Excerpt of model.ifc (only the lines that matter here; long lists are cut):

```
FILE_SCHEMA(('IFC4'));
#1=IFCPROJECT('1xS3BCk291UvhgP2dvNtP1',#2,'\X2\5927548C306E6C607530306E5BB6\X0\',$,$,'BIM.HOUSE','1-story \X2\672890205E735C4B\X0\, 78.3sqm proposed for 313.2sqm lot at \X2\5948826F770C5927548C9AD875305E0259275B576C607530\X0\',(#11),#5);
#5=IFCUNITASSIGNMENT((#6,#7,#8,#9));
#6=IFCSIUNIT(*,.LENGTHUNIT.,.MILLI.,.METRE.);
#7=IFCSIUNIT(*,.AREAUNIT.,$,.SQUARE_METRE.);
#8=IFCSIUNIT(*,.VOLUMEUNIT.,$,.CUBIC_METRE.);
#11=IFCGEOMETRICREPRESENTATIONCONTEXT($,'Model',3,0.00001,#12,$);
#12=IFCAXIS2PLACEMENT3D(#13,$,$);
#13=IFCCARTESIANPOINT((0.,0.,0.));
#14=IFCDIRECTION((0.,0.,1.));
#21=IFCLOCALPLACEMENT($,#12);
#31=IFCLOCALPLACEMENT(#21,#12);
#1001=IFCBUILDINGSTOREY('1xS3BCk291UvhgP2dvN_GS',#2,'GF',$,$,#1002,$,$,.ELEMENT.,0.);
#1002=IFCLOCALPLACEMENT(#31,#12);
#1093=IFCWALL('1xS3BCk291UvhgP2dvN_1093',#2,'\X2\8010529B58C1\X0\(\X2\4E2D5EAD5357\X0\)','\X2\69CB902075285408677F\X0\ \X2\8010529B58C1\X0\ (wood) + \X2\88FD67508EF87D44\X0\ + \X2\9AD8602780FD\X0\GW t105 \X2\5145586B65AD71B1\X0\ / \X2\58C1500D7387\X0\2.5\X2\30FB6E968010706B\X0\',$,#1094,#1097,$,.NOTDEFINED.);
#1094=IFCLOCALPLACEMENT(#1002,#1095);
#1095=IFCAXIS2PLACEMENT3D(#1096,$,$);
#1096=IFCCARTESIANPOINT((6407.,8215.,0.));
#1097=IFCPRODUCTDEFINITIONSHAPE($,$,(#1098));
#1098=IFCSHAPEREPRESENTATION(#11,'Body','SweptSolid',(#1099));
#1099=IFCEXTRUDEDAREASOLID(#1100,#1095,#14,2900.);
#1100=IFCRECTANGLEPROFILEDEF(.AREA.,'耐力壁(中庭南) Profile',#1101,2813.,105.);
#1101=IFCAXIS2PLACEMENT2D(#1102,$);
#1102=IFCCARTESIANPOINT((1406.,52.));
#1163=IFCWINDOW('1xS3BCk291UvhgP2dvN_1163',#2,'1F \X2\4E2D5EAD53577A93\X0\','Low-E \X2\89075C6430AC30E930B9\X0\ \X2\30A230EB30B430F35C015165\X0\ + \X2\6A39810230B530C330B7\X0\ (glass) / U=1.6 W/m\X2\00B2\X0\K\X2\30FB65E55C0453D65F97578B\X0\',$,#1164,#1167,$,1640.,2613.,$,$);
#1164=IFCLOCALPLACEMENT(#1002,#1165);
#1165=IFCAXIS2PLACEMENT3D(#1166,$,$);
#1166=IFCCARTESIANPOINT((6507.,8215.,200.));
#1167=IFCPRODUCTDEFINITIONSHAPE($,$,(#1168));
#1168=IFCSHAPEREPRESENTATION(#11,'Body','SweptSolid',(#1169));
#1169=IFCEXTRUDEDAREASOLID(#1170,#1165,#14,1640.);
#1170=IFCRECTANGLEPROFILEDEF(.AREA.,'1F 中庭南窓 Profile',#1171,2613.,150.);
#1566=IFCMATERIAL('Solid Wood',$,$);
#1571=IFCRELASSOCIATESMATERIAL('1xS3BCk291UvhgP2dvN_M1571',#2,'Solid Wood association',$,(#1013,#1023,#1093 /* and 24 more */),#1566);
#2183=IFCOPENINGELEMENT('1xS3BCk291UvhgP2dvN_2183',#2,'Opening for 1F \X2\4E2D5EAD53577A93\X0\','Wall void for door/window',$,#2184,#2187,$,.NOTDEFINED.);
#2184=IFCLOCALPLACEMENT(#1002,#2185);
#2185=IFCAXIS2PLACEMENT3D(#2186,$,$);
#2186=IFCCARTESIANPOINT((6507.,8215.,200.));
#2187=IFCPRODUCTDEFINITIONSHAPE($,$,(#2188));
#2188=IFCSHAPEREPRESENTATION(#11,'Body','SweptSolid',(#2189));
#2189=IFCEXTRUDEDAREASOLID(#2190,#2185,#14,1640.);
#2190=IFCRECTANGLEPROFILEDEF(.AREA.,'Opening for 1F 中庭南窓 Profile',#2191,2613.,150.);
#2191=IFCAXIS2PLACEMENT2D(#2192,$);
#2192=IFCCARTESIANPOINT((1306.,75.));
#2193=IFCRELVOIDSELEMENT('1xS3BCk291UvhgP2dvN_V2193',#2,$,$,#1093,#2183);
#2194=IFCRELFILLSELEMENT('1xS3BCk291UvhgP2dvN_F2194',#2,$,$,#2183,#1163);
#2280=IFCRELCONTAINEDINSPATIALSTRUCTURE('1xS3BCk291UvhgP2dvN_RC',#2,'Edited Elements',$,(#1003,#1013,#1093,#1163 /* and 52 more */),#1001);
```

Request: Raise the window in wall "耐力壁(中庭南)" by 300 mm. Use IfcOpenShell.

```python
import numpy as np
import ifcopenshell
import ifcopenshell.api.geometry
import ifcopenshell.util.placement
import ifcopenshell.util.unit

model = ifcopenshell.open("model.ifc")
unit_scale = ifcopenshell.util.unit.calculate_unit_scale(model)

window = model.by_guid("1xS3BCk291UvhgP2dvN_1163")
opening = window.FillsVoids[0].RelatingOpeningElement
dz = 0.3 / unit_scale

shift = np.array([0.0, 0.0, dz])
# The window is not placed relative to its opening, so move both.
for product in (opening, window):
    matrix = ifcopenshell.util.placement.get_local_placement(product.ObjectPlacement)
    matrix[:3, 3] += shift
    ifcopenshell.api.geometry.edit_object_placement(model, product=product, matrix=matrix, is_si=False)

print(f"moved by {dz * unit_scale:+.3f} m")

model.write("model_v2.ifc")
```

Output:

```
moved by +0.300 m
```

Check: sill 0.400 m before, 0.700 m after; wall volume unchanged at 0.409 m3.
